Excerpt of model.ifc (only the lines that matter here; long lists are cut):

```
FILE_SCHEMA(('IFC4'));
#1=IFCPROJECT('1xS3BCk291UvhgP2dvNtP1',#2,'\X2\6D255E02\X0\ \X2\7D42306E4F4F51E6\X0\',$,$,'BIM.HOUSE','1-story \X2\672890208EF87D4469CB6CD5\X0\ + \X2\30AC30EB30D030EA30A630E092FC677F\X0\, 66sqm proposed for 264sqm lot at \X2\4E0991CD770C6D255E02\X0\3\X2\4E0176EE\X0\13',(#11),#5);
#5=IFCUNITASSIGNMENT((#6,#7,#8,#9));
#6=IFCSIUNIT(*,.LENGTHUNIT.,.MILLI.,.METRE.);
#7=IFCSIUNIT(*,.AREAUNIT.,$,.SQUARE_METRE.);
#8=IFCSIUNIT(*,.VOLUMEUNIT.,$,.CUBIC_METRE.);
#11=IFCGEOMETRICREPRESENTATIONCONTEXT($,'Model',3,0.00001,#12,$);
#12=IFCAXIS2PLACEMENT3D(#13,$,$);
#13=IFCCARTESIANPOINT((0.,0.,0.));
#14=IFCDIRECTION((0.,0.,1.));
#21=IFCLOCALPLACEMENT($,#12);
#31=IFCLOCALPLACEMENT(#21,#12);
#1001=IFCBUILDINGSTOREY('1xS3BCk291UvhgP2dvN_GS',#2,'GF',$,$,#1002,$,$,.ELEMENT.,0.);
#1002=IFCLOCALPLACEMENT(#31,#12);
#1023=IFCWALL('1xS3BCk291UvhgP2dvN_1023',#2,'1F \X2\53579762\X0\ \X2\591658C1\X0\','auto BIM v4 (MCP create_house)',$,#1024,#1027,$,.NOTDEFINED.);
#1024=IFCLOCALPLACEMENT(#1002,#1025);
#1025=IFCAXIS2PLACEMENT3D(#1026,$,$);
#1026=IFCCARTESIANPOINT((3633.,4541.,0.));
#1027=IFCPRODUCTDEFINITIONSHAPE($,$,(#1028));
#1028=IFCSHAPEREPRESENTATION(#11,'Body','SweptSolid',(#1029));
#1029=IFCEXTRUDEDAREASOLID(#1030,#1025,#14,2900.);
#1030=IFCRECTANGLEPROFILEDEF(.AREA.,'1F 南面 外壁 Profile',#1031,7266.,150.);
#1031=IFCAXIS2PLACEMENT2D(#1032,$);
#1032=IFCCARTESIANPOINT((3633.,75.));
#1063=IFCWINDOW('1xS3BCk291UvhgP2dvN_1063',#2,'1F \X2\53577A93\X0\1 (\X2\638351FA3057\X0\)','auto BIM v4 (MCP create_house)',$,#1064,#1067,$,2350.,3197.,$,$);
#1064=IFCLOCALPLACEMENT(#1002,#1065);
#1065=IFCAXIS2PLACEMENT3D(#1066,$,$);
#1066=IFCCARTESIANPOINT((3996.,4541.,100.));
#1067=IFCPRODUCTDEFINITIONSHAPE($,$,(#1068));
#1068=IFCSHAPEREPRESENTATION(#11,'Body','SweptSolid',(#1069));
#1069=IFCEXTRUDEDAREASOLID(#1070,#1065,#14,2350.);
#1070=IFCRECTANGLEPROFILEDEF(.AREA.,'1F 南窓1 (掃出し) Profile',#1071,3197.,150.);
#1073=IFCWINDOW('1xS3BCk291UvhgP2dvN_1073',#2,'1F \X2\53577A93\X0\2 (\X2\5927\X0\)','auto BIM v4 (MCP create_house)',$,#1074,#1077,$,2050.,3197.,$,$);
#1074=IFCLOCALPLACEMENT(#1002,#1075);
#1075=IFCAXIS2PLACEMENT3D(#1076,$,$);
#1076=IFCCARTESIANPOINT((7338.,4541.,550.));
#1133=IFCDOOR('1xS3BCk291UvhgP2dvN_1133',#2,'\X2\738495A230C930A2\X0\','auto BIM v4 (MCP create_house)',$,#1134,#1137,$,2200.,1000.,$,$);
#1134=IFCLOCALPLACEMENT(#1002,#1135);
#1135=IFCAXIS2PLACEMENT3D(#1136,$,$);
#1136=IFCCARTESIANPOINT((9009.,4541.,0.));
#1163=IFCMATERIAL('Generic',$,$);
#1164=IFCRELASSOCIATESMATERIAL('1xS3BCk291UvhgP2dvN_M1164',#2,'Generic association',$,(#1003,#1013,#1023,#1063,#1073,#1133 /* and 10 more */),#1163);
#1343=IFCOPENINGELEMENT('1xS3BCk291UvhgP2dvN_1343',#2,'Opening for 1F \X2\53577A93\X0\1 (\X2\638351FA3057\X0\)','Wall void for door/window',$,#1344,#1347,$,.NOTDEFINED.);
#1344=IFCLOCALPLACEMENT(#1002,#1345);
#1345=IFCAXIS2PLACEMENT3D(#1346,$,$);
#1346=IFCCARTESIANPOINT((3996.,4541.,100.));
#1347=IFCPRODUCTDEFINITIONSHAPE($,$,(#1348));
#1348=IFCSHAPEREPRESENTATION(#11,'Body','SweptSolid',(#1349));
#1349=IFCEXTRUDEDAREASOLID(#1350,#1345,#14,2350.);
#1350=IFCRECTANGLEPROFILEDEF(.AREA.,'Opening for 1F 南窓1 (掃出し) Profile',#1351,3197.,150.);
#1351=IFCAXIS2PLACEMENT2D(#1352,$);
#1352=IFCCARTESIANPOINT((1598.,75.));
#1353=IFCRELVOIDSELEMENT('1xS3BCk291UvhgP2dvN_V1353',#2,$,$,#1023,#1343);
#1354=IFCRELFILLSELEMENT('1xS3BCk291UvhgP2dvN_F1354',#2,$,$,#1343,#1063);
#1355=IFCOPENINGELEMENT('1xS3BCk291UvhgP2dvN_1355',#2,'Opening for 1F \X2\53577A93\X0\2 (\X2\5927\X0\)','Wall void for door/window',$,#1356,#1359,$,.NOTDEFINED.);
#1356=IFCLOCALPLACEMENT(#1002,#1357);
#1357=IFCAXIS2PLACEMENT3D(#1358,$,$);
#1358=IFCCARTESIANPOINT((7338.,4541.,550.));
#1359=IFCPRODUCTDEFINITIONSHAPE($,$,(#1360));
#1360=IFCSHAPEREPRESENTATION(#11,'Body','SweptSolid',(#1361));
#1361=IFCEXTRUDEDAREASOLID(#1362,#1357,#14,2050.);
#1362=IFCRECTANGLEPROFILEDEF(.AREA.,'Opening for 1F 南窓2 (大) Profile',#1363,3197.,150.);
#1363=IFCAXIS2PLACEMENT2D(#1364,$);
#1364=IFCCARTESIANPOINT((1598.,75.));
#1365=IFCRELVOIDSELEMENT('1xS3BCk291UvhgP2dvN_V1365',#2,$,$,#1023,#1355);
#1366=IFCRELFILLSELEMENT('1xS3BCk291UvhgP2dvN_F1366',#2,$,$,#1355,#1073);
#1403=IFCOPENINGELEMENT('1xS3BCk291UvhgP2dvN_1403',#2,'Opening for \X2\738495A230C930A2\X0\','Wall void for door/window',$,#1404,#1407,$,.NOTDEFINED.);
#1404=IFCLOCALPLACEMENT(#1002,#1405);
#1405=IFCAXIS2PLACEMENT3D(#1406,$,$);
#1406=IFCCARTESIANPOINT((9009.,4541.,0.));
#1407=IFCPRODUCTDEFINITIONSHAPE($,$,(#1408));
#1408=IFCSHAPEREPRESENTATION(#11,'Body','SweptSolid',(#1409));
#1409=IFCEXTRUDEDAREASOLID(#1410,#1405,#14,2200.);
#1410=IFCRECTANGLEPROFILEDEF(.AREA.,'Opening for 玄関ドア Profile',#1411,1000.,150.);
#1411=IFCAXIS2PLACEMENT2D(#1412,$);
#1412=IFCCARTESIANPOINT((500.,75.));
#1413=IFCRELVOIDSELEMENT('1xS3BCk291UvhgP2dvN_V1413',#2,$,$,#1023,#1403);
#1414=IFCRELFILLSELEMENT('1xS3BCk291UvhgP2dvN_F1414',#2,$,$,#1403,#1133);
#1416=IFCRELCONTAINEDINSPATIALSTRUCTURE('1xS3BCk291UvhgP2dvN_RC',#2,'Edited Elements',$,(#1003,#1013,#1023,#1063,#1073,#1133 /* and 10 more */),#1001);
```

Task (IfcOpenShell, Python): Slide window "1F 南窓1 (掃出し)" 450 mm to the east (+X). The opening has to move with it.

```python
import ifcopenshell
import ifcopenshell.api.geometry
import ifcopenshell.util.placement

model = ifcopenshell.open("model.ifc")

window = model.by_guid("1xS3BCk291UvhgP2dvN_1063")
opening = window.FillsVoids[0].RelatingOpeningElement
wall = opening.VoidsElements[0].RelatingBuildingElement

wall_matrix = ifcopenshell.util.placement.get_local_placement(wall.ObjectPlacement)
shift = wall_matrix[:3, 0] * 450.0
before = ifcopenshell.util.placement.get_local_placement(window.ObjectPlacement)[:3, 3].copy()

# The window is not placed relative to its opening, so move both.
for product in (opening, window):
    matrix = ifcopenshell.util.placement.get_local_placement(product.ObjectPlacement)
    matrix[:3, 3] += shift
    ifcopenshell.api.geometry.edit_object_placement(model, product=product, matrix=matrix, is_si=False)

after = ifcopenshell.util.placement.get_local_placement(window.ObjectPlacement)[:3, 3]
print("window moved by", (after - before).round(3) + 0.0)

model.write("model-out.ifc")
```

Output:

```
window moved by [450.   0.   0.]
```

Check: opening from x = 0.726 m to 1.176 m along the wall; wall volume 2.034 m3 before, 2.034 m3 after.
